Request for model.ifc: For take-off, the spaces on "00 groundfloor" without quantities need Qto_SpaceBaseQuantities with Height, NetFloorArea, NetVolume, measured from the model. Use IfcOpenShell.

First a look at what the model holds.

```python
import ifcopenshell
import ifcopenshell.util.element
import ifcopenshell.util.unit

model = ifcopenshell.open("model.ifc")
print(model.schema)
for unit_type in ("LENGTHUNIT", "AREAUNIT", "VOLUMEUNIT"):
    print(unit_type, ifcopenshell.util.unit.calculate_unit_scale(model, unit_type))
storey = next(s for s in model.by_type("IfcBuildingStorey") if s.Name == "00 groundfloor")
spaces = [e for e in ifcopenshell.util.element.get_decomposition(storey) if e.is_a("IfcSpace")]
for e in sorted(spaces, key=lambda e: e.id()):
    print(e.id(), e.is_a(), e.Name, list(ifcopenshell.util.element.get_psets(e, qtos_only=True)), sep=" | ")
```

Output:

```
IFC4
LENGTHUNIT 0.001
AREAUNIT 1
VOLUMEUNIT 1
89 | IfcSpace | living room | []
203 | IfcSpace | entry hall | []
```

```python
import ifcopenshell
import ifcopenshell.api.pset
import ifcopenshell.geom
import ifcopenshell.util.element
import ifcopenshell.util.shape
import ifcopenshell.util.unit

model = ifcopenshell.open("model.ifc")
unit_scale = ifcopenshell.util.unit.calculate_unit_scale(model)
area_scale = ifcopenshell.util.unit.calculate_unit_scale(model, "AREAUNIT")
volume_scale = ifcopenshell.util.unit.calculate_unit_scale(model, "VOLUMEUNIT")
settings = ifcopenshell.geom.settings()

storey = next(s for s in model.by_type("IfcBuildingStorey") if s.Name == "00 groundfloor")
spaces = [e for e in ifcopenshell.util.element.get_decomposition(storey) if e.is_a("IfcSpace")]

for e in sorted(spaces, key=lambda e: e.id()):
    if ifcopenshell.util.element.get_psets(e, qtos_only=True, should_inherit=False):
        continue
    # Geometry comes back in metres, in the element's own axes.
    shape = ifcopenshell.geom.create_shape(settings, e)
    values = {
        "Height": ifcopenshell.util.shape.get_z(shape.geometry) / unit_scale,
        "NetFloorArea": ifcopenshell.util.shape.get_footprint_area(shape.geometry) / area_scale,
        "NetVolume": ifcopenshell.util.shape.get_volume(shape.geometry) / volume_scale,
    }
    qto = ifcopenshell.api.pset.add_qto(model, product=e, name="Qto_SpaceBaseQuantities")
    ifcopenshell.api.pset.edit_qto(model, qto=qto, properties=values)
    print(e.id(), {k: round(v, 3) for k, v in values.items()})

model.write("model_updated.ifc")
```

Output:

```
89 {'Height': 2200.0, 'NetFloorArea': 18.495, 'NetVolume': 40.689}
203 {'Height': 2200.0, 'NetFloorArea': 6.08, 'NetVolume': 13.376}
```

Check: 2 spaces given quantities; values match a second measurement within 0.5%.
